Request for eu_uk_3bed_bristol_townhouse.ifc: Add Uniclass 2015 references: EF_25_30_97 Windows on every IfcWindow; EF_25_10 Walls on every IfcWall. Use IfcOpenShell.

First a look at what the model holds.

```python
import ifcopenshell

model = ifcopenshell.open("eu_uk_3bed_bristol_townhouse.ifc")
print(model.schema)
print("classifications:", [c.Name for c in model.by_type("IfcClassification")])
for ifc_class in ("IfcDoor", "IfcRoof", "IfcStair", "IfcWall", "IfcWindow"):
    print(ifc_class, len(model.by_type(ifc_class)))
```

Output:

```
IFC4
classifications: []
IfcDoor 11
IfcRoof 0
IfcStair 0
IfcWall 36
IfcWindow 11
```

```python
import ifcopenshell
import ifcopenshell.api.classification

model = ifcopenshell.open("eu_uk_3bed_bristol_townhouse.ifc")

system = ifcopenshell.api.classification.add_classification(model, classification="Uniclass 2015")

codes = {
    "IfcWindow": ("EF_25_30_97", "Windows"),
    "IfcWall": ("EF_25_10", "Walls"),
}
for ifc_class, (code, name) in codes.items():
    products = model.by_type(ifc_class)
    ifcopenshell.api.classification.add_reference(
        model, products=products, classification=system, identification=code, name=name
    )
    print(code, len(products))

model.write("eu_uk_3bed_bristol_townhouse_rev.ifc")
```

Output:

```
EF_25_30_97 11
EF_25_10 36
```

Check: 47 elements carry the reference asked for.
